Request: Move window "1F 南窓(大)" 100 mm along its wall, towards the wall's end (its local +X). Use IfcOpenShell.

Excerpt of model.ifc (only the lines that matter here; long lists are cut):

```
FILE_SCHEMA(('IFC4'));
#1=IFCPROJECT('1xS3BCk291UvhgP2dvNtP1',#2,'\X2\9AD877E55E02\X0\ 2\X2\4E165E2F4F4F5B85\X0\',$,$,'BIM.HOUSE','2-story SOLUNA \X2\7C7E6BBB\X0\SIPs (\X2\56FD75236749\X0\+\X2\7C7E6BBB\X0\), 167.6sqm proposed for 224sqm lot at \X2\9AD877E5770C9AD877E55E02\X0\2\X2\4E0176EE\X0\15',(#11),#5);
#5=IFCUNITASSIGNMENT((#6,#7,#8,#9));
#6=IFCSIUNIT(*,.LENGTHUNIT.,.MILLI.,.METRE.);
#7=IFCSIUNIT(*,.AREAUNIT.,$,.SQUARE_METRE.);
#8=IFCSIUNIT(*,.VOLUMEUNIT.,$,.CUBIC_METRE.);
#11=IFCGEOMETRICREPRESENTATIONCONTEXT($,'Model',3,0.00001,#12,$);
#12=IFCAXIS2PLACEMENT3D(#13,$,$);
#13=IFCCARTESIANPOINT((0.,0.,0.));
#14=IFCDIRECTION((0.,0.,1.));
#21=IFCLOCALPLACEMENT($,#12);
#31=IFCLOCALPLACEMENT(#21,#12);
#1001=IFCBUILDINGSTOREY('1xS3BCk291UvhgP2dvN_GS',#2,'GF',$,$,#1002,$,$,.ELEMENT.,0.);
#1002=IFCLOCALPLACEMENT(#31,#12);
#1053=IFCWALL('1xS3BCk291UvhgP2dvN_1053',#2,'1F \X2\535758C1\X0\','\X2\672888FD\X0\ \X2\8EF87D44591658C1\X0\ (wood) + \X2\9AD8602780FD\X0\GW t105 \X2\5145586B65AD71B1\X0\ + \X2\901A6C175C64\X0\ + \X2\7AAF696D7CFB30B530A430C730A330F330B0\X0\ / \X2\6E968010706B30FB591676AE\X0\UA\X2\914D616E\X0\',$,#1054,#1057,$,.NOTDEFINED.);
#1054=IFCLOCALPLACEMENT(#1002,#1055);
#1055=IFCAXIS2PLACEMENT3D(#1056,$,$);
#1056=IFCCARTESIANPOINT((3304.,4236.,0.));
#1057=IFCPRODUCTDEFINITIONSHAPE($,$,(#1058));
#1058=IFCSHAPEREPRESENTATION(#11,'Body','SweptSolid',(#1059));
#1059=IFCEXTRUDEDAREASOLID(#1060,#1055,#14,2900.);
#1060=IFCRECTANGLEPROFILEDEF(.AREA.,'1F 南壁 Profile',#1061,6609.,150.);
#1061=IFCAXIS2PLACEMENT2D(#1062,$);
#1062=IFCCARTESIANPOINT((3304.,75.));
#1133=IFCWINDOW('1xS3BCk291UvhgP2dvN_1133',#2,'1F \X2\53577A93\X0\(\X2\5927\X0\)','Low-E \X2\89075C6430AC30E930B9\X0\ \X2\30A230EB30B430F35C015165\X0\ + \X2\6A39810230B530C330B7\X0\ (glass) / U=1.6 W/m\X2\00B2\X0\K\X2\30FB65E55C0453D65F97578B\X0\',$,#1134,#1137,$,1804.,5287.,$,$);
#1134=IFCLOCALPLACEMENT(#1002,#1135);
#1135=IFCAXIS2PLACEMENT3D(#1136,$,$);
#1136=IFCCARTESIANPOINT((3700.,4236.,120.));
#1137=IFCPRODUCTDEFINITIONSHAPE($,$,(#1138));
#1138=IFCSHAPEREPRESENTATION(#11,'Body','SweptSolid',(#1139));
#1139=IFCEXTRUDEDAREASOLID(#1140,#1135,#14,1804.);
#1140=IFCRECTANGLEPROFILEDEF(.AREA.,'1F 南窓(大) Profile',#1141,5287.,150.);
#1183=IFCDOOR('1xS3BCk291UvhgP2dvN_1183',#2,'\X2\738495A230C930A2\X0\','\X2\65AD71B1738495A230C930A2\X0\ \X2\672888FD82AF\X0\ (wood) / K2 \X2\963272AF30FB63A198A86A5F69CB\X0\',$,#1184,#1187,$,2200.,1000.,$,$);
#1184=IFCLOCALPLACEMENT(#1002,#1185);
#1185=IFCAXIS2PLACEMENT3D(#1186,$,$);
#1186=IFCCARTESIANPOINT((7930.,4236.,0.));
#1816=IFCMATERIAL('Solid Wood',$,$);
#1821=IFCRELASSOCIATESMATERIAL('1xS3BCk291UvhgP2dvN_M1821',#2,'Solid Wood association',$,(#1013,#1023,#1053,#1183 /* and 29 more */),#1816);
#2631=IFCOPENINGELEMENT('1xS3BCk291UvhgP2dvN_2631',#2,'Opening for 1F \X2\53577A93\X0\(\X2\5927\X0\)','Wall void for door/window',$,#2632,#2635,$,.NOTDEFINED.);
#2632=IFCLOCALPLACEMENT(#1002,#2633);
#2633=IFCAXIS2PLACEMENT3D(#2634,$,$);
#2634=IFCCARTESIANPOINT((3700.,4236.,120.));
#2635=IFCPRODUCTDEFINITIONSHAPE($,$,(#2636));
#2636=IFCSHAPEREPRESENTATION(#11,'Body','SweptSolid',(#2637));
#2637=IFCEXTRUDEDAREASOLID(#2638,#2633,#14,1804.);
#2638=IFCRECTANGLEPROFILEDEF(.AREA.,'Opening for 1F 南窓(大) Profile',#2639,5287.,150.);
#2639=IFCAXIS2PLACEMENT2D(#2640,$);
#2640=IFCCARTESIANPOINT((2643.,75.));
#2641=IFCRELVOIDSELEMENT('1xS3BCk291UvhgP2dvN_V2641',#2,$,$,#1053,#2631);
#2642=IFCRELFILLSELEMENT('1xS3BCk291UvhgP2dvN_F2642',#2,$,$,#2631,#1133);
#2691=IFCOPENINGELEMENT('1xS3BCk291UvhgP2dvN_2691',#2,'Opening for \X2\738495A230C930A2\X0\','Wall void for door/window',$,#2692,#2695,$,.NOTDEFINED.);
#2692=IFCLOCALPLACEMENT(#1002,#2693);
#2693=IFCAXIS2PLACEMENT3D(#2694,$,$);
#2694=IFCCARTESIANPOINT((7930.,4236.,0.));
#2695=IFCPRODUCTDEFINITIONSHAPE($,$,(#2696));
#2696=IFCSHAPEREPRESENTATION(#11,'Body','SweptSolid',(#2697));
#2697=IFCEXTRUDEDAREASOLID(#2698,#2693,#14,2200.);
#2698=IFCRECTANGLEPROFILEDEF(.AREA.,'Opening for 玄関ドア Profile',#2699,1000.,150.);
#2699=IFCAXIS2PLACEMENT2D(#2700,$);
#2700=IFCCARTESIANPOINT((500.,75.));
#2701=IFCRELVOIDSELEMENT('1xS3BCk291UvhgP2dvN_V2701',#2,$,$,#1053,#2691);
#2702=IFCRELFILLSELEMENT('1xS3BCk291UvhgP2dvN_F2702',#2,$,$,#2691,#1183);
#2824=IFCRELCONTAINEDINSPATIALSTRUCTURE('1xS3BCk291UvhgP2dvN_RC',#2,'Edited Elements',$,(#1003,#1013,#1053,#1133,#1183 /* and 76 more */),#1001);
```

```python
import ifcopenshell
import ifcopenshell.api.geometry
import ifcopenshell.util.placement

model = ifcopenshell.open("model.ifc")

window = model.by_guid("1xS3BCk291UvhgP2dvN_1133")
opening = window.FillsVoids[0].RelatingOpeningElement
wall = opening.VoidsElements[0].RelatingBuildingElement

wall_matrix = ifcopenshell.util.placement.get_local_placement(wall.ObjectPlacement)
shift = wall_matrix[:3, 0] * 100.0
before = ifcopenshell.util.placement.get_local_placement(window.ObjectPlacement)[:3, 3].copy()

# The window is not placed relative to its opening, so move both.
for product in (opening, window):
    matrix = ifcopenshell.util.placement.get_local_placement(product.ObjectPlacement)
    matrix[:3, 3] += shift
    ifcopenshell.api.geometry.edit_object_placement(model, product=product, matrix=matrix, is_si=False)

after = ifcopenshell.util.placement.get_local_placement(window.ObjectPlacement)[:3, 3]
print("window moved by", (after - before).round(3) + 0.0)

model.write("model_v2.ifc")
```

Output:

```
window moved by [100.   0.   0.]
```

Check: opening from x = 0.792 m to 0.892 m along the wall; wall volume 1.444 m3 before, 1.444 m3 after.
